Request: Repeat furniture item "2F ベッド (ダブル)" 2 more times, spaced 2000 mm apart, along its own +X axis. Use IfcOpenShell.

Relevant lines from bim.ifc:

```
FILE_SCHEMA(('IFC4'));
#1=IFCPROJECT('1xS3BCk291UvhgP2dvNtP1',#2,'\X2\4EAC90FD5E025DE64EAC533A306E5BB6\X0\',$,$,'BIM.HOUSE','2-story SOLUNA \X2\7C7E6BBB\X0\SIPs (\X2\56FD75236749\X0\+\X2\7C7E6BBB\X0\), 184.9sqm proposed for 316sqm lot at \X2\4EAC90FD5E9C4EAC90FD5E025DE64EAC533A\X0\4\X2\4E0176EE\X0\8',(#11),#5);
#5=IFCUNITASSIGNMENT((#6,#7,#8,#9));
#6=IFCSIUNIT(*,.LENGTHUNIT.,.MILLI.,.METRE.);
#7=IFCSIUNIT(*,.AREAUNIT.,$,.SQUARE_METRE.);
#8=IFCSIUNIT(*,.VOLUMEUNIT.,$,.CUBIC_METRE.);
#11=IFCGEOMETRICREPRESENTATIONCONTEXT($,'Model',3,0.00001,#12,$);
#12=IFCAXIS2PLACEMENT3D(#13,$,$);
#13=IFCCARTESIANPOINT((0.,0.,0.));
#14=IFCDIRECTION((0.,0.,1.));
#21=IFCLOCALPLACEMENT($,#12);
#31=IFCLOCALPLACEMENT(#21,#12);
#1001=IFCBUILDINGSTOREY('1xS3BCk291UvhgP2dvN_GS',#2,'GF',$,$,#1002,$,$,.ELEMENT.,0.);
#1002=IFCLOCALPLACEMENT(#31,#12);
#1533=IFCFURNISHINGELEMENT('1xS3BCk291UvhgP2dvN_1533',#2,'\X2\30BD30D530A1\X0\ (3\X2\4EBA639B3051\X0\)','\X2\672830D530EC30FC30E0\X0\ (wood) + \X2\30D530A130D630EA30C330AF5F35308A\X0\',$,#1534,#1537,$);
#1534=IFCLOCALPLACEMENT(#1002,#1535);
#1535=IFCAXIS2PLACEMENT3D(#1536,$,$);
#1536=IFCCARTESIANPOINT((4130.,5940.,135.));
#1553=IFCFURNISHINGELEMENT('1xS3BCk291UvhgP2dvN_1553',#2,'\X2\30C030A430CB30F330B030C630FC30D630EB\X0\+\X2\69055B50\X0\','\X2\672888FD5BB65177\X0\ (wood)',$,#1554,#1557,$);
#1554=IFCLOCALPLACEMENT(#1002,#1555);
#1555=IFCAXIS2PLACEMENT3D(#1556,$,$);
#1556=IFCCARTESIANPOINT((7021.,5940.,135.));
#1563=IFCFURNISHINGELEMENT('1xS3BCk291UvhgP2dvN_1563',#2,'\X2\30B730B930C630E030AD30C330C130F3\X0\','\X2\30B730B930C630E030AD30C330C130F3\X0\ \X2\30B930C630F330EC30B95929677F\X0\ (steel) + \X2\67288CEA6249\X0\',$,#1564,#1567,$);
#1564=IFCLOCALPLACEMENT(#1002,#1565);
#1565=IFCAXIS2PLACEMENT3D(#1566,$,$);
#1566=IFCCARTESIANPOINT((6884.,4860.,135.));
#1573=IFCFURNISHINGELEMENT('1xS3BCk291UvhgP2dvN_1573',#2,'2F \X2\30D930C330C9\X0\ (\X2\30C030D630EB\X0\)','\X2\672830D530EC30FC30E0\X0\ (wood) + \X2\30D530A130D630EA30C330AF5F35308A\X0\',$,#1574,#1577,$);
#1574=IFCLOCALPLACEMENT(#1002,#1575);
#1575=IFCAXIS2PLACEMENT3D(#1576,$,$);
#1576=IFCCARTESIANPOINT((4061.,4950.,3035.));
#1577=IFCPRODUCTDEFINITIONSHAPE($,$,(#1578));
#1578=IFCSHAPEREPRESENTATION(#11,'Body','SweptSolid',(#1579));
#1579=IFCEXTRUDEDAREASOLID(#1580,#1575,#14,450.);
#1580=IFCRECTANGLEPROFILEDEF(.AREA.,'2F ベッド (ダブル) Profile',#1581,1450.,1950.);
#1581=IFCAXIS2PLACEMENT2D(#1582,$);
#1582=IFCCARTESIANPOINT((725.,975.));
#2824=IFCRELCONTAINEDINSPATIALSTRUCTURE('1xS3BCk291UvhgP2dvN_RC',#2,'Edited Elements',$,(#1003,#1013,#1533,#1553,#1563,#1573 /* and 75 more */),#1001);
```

```python
import ifcopenshell
import ifcopenshell.api.geometry
import ifcopenshell.api.root
import ifcopenshell.util.element
import ifcopenshell.util.placement
import ifcopenshell.util.unit

model = ifcopenshell.open("bim.ifc")
unit_scale = ifcopenshell.util.unit.calculate_unit_scale(model)


def reuse_history(source, copy):
    """copy_class also copies each property set's owner history, people and application; keep the originals."""
    for rel in copy.IsDefinedBy:
        if rel.is_a("IfcRelDefinesByProperties") and (history := rel.RelatingPropertyDefinition.OwnerHistory):
            rel.RelatingPropertyDefinition.OwnerHistory = source.OwnerHistory
            ifcopenshell.util.element.remove_deep2(model, history)


source = model.by_guid("1xS3BCk291UvhgP2dvN_1573")
base = ifcopenshell.util.placement.get_local_placement(source.ObjectPlacement)
step = base[:3, 0] * 2 / unit_scale

for i in range(1, 3):
    copy = ifcopenshell.api.root.copy_class(model, product=source)
    copy.Representation = ifcopenshell.util.element.copy_deep(
        model, source.Representation, exclude=["IfcGeometricRepresentationContext", "IfcRepresentationMap"]
    )
    reuse_history(source, copy)
    matrix = base.copy()
    matrix[:3, 3] += i * step
    print("added at", matrix[:3, 3].round(3) + 0.0)
    ifcopenshell.api.geometry.edit_object_placement(model, product=copy, matrix=matrix, is_si=False)

model.write("bim-out.ifc")
```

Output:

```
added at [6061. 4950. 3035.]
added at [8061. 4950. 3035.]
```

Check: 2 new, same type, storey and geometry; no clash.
